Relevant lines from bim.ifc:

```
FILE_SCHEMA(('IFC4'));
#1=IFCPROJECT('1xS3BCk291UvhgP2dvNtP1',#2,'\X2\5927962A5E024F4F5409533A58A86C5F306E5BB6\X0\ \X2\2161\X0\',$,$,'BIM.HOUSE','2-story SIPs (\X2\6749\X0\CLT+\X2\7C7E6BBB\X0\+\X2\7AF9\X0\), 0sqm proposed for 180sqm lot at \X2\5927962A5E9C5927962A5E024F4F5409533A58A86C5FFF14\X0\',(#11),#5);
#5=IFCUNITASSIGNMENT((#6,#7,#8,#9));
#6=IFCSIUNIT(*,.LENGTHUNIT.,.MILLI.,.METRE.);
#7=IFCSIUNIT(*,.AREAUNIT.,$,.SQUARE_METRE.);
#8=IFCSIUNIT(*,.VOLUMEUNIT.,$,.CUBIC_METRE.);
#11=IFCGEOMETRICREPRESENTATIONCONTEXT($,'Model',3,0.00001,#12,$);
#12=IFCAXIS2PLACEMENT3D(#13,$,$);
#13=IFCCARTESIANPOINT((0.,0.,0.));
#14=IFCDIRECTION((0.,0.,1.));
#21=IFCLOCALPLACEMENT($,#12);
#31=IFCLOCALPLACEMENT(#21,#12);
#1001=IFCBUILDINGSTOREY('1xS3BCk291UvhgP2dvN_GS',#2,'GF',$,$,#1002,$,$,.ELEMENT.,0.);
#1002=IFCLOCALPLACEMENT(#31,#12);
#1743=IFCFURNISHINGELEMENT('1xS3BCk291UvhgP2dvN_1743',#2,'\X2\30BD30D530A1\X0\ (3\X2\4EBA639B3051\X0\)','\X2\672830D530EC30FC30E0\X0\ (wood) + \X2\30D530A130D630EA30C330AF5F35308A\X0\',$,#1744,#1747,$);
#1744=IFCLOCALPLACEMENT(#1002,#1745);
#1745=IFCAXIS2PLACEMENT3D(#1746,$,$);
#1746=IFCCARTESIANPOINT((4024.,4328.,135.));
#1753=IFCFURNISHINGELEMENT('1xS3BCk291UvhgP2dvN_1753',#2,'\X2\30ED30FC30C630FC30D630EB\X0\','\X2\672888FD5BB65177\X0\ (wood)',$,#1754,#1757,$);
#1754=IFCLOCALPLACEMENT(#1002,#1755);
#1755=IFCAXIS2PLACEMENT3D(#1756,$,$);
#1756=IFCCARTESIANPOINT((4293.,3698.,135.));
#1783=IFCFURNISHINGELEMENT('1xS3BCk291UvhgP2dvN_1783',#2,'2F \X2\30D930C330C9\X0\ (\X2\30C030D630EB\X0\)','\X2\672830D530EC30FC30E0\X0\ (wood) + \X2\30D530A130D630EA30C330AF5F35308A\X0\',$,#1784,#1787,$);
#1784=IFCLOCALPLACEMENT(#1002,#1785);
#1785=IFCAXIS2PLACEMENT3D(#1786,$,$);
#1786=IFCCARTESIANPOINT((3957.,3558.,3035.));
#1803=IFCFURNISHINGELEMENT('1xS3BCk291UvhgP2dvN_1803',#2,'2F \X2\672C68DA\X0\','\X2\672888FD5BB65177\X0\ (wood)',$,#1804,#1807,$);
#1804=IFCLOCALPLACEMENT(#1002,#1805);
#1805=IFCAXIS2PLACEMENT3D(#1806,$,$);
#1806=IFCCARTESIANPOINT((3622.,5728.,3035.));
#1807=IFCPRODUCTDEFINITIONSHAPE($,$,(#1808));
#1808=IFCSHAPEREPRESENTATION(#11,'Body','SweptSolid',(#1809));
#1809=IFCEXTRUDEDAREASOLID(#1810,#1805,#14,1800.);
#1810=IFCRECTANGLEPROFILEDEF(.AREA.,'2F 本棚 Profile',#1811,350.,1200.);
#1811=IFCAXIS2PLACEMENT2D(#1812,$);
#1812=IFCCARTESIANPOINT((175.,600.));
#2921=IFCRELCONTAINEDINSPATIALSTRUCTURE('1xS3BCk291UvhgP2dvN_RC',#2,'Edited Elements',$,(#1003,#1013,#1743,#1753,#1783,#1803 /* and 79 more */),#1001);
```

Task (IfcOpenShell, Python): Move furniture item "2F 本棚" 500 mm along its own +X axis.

```python
import ifcopenshell
import ifcopenshell.api.geometry
import ifcopenshell.util.placement
import ifcopenshell.util.unit

model = ifcopenshell.open("bim.ifc")
unit_scale = ifcopenshell.util.unit.calculate_unit_scale(model)

item = model.by_guid("1xS3BCk291UvhgP2dvN_1803")
matrix = ifcopenshell.util.placement.get_local_placement(item.ObjectPlacement)
matrix[:3, 3] += matrix[:3, 0] * 0.5 / unit_scale
ifcopenshell.api.geometry.edit_object_placement(model, product=item, matrix=matrix, is_si=False)

print(ifcopenshell.util.placement.get_local_placement(item.ObjectPlacement).round(3) + 0.0)

model.write("bim_v2.ifc")
```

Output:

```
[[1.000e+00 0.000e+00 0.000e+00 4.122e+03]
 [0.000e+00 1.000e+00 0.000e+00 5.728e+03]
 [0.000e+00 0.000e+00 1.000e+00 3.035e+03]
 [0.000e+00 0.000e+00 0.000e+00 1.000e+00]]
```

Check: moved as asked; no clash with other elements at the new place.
